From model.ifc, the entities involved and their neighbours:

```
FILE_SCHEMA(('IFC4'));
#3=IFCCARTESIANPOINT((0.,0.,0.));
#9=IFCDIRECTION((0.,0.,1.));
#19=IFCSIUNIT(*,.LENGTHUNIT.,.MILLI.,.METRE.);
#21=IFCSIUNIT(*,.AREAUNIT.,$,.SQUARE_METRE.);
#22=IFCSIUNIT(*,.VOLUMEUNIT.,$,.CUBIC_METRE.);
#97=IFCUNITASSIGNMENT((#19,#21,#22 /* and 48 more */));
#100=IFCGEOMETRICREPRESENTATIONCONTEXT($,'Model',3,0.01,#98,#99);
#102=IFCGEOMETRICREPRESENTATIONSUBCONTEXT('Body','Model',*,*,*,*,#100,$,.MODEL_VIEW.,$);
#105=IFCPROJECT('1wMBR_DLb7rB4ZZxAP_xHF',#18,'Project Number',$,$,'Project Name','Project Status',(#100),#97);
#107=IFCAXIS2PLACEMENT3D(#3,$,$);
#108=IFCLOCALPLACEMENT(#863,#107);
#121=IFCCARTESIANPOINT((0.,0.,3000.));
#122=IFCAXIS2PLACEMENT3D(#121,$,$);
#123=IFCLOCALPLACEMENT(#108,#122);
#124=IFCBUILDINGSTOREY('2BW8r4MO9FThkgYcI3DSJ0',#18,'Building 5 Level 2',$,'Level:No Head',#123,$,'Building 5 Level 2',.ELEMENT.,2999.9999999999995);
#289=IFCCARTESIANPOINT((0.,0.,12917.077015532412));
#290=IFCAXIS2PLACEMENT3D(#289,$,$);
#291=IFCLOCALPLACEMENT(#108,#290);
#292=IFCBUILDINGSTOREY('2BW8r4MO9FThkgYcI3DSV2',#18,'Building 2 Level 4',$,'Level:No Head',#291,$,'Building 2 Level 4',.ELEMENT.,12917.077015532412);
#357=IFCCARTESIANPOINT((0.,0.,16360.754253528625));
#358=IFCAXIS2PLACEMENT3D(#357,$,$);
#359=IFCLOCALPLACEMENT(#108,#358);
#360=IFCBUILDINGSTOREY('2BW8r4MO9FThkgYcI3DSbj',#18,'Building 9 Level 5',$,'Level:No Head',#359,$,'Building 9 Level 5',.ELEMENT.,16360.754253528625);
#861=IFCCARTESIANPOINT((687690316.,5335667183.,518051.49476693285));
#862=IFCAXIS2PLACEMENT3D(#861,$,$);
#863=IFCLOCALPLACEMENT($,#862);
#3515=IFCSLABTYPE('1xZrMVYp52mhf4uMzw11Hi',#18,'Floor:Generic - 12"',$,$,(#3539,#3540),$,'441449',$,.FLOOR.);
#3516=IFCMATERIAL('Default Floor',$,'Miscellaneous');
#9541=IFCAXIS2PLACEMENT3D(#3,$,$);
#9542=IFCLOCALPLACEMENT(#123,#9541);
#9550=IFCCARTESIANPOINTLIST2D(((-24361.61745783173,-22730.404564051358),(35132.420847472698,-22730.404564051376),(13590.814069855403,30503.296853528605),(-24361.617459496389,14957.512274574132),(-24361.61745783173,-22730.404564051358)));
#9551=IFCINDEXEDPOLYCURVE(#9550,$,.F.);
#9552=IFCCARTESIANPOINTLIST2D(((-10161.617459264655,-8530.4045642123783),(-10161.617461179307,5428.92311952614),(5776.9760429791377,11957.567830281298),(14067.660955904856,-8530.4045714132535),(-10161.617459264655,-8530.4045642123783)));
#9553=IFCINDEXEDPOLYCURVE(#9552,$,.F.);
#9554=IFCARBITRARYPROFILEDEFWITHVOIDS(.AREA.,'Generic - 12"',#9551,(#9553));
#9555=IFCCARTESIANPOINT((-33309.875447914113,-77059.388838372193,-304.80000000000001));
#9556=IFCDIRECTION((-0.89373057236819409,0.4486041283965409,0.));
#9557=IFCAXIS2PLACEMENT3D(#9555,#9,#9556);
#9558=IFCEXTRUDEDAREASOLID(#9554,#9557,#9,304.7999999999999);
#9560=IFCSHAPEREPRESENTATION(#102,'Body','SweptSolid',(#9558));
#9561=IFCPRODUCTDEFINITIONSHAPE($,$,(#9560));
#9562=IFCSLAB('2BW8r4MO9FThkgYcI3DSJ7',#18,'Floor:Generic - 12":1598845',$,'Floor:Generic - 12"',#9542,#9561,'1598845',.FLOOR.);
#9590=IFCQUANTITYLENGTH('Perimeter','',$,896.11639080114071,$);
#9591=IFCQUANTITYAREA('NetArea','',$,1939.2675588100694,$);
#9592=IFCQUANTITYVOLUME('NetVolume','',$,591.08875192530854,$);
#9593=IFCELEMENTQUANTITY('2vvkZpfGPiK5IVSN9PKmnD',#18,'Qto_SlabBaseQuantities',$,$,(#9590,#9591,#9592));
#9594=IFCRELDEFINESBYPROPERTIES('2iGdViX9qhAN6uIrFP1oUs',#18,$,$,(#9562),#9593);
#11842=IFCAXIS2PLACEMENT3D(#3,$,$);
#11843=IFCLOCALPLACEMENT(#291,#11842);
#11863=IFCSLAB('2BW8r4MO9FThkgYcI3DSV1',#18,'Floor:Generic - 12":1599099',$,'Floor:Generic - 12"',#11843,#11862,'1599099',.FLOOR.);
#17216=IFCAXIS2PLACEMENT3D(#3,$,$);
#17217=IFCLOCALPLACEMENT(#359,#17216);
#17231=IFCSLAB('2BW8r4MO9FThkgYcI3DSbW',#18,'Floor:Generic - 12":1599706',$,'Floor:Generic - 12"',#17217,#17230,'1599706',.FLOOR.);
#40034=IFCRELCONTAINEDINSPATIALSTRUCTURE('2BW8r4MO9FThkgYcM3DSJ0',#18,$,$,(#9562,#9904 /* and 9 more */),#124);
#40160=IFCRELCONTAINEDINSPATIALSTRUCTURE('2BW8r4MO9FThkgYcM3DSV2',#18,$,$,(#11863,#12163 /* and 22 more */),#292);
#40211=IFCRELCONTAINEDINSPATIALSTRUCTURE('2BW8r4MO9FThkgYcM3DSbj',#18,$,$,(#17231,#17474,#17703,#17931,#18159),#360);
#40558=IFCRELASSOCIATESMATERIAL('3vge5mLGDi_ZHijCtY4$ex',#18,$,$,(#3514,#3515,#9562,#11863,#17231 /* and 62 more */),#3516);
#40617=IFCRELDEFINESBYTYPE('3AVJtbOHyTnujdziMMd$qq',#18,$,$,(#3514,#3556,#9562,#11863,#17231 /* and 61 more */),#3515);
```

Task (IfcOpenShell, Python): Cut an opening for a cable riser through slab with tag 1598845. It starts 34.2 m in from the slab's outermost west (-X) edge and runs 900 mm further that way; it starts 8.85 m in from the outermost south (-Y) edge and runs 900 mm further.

```python
import numpy as np
import ifcopenshell
import ifcopenshell.api.feature
import ifcopenshell.api.geometry
import ifcopenshell.api.pset
import ifcopenshell.api.root
import ifcopenshell.geom
import ifcopenshell.util.element
import ifcopenshell.util.placement
import ifcopenshell.util.representation
import ifcopenshell.util.shape
import ifcopenshell.util.unit

model = ifcopenshell.open("model.ifc")
unit_scale = ifcopenshell.util.unit.calculate_unit_scale(model)
area_scale = ifcopenshell.util.unit.calculate_unit_scale(model, "AREAUNIT")
volume_scale = ifcopenshell.util.unit.calculate_unit_scale(model, "VOLUMEUNIT")
settings = ifcopenshell.geom.settings()


def volume(element):
    """Net volume in cubic metres, openings subtracted."""
    shape = ifcopenshell.geom.create_shape(settings, element)
    return ifcopenshell.util.shape.get_volume(shape.geometry)


slab = model.by_guid("2BW8r4MO9FThkgYcI3DSJ7")
before = volume(slab)

# Extent in the slab's own axes, in metres. The edges named are its -X and -Y sides.
slab_shape = ifcopenshell.geom.create_shape(settings, slab)
vertices = ifcopenshell.util.shape.get_vertices(slab_shape.geometry)
x_min, y_min, bottom = vertices.min(axis=0)
top = vertices[:, 2].max()

opening = ifcopenshell.api.root.create_entity(model, ifc_class="IfcOpeningElement", name="Cable riser opening", predefined_type="OPENING")
context = ifcopenshell.util.representation.get_context(model, "Model", "Body", "MODEL_VIEW")
width, depth = 0.9, 0.9
outline = [(0.0, 0.0), (width, 0.0), (width, depth), (0.0, depth), (0.0, 0.0)]
# Overshoot both faces by 50 mm so the cut is clean.
shape = ifcopenshell.api.geometry.add_slab_representation(
    model, context=context, depth=top - bottom + 0.1, polyline=outline
)
ifcopenshell.api.geometry.assign_representation(model, product=opening, representation=shape)

matrix = ifcopenshell.util.placement.get_local_placement(slab.ObjectPlacement)
matrix[:, 3] = matrix @ np.append(np.array([x_min + 34.2, y_min + 8.85, bottom - 0.05]) / unit_scale, 1.0)
ifcopenshell.api.geometry.edit_object_placement(model, product=opening, matrix=matrix, is_si=False)
ifcopenshell.api.feature.add_feature(model, feature=opening, element=slab)

after = volume(slab)

# Update the slab's stored quantities.
qto = model.by_id(ifcopenshell.util.element.get_pset(slab, "Qto_SlabBaseQuantities", should_inherit=False)["id"])
ifcopenshell.api.pset.edit_qto(model, qto=qto, properties={
    "NetArea": after / (top - bottom) / area_scale,
    "NetVolume": after / volume_scale,
})

print(f"slab volume {before:.3f} -> {after:.3f} m3")

model.write("model_updated.ifc")
```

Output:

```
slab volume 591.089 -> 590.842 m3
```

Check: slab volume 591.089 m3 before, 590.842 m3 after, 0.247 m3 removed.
